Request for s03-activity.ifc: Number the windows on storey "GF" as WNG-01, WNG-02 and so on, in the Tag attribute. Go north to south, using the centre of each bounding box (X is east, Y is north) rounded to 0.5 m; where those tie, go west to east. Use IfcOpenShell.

First a look at what the model holds.

```python
import ifcopenshell
import ifcopenshell.util.element
import ifcopenshell.util.placement

model = ifcopenshell.open("s03-activity.ifc")
print(model.schema)
storey = next(s for s in model.by_type("IfcBuildingStorey") if s.Name == "GF")
windows = [e for e in ifcopenshell.util.element.get_decomposition(storey) if e.is_a("IfcWindow")]
for e in sorted(windows, key=lambda e: e.id()):
    origin = ifcopenshell.util.placement.get_local_placement(e.ObjectPlacement)[:3, 3]
    print(e.id(), e.Tag, e.Name, origin.round(2) + 0.0, sep=" | ")
```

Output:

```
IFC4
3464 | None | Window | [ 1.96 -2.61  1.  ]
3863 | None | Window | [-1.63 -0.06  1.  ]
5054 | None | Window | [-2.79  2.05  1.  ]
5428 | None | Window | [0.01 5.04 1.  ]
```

```python
import ifcopenshell
import ifcopenshell.geom
import ifcopenshell.util.element
import ifcopenshell.util.shape

model = ifcopenshell.open("s03-activity.ifc")
settings = ifcopenshell.geom.settings()
settings.set("use-world-coords", True)


def centre(element):
    shape = ifcopenshell.geom.create_shape(settings, element)
    return ifcopenshell.util.shape.get_bbox_centroid(shape.geometry)


storey = next(s for s in model.by_type("IfcBuildingStorey") if s.Name == "GF")
windows = [e for e in ifcopenshell.util.element.get_decomposition(storey) if e.is_a("IfcWindow")]

# Insertion points can sit at a corner or the storey origin, so sort by the geometry (in metres).
centres = {e: centre(e) for e in windows}
windows.sort(key=lambda e: (-round(centres[e][1] / 0.5), centres[e][0]))

for i, e in enumerate(windows, start=1):
    number = f"WNG-{i:02d}"
    e.Tag = number
    print(e.id(), number)

model.write("s03-activity_v2.ifc")
```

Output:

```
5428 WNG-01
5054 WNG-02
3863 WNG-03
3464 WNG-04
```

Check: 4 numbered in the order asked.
